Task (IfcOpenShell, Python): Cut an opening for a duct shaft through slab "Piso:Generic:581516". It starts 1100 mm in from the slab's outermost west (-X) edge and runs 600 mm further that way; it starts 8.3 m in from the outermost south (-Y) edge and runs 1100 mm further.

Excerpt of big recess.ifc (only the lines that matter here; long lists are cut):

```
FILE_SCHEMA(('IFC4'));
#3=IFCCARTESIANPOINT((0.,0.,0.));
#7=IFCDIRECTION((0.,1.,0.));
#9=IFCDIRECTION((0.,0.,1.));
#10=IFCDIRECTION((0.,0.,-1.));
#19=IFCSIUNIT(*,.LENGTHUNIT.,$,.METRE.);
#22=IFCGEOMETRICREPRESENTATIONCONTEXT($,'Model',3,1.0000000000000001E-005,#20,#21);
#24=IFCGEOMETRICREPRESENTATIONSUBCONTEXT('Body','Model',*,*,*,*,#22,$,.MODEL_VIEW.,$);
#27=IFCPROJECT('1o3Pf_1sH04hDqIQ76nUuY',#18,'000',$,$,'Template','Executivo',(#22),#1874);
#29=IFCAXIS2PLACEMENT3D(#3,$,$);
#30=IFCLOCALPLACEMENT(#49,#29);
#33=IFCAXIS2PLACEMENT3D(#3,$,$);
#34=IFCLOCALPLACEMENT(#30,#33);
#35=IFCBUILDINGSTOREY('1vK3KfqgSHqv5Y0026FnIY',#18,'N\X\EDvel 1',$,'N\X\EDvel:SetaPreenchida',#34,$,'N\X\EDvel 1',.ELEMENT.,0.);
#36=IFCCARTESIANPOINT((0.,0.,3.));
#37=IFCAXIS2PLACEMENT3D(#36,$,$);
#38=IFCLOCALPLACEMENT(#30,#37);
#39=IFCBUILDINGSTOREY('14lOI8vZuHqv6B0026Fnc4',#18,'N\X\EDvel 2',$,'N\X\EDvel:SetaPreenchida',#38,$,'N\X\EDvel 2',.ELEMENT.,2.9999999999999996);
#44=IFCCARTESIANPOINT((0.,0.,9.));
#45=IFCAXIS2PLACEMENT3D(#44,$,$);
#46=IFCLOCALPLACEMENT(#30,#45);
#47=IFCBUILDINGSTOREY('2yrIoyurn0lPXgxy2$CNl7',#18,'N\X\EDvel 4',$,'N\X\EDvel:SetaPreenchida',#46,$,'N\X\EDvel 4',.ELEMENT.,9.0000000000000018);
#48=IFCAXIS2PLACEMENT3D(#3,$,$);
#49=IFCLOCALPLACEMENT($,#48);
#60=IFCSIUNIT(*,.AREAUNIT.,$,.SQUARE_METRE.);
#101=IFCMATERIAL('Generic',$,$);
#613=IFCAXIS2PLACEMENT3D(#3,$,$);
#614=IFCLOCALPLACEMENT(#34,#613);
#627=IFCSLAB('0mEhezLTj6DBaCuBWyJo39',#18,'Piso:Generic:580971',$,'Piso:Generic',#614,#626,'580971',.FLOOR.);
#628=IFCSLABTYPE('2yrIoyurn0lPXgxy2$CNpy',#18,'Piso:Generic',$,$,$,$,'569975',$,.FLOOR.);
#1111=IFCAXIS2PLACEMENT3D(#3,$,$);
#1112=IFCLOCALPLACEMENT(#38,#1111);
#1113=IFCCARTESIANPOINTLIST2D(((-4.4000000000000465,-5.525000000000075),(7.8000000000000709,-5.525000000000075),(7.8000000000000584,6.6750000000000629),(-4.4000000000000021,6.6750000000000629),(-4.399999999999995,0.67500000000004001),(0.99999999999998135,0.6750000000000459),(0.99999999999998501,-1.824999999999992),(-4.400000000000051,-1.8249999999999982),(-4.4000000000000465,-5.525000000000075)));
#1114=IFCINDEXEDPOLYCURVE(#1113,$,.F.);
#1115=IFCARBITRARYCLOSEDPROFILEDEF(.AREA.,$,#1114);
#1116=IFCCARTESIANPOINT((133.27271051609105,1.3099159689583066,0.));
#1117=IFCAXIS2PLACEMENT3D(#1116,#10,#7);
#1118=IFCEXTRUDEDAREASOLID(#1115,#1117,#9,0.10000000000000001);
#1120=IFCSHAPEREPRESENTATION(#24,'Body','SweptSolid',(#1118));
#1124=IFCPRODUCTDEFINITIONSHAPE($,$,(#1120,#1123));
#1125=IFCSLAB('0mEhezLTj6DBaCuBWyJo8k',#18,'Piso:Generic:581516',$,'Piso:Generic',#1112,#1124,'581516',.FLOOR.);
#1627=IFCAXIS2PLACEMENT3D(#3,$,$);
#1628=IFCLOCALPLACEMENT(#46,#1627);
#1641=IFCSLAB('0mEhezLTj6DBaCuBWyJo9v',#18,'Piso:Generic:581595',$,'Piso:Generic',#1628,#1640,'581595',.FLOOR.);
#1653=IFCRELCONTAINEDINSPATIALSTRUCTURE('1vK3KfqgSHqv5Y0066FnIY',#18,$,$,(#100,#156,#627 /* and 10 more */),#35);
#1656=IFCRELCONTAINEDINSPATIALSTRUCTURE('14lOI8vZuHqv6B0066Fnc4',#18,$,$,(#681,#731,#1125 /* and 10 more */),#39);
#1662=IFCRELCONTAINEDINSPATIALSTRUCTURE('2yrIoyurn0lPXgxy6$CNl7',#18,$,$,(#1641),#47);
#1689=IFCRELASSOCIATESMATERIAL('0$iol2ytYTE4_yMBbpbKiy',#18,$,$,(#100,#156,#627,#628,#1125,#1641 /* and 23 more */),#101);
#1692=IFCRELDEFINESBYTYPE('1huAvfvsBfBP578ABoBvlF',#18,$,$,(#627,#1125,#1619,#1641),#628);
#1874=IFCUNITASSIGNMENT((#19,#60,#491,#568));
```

```python
import numpy as np
import ifcopenshell
import ifcopenshell.api.feature
import ifcopenshell.api.geometry
import ifcopenshell.api.root
import ifcopenshell.geom
import ifcopenshell.util.placement
import ifcopenshell.util.representation
import ifcopenshell.util.shape
import ifcopenshell.util.unit

model = ifcopenshell.open("big recess.ifc")
unit_scale = ifcopenshell.util.unit.calculate_unit_scale(model)
settings = ifcopenshell.geom.settings()


def volume(element):
    """Net volume in cubic metres, openings subtracted."""
    shape = ifcopenshell.geom.create_shape(settings, element)
    return ifcopenshell.util.shape.get_volume(shape.geometry)


slab = model.by_guid("0mEhezLTj6DBaCuBWyJo8k")
before = volume(slab)

# Extent in the slab's own axes, in metres. The edges named are its -X and -Y sides.
slab_shape = ifcopenshell.geom.create_shape(settings, slab)
vertices = ifcopenshell.util.shape.get_vertices(slab_shape.geometry)
x_min, y_min, bottom = vertices.min(axis=0)
top = vertices[:, 2].max()

opening = ifcopenshell.api.root.create_entity(model, ifc_class="IfcOpeningElement", name="Duct shaft opening", predefined_type="OPENING")
context = ifcopenshell.util.representation.get_context(model, "Model", "Body", "MODEL_VIEW")
width, depth = 0.6, 1.1
outline = [(0.0, 0.0), (width, 0.0), (width, depth), (0.0, depth), (0.0, 0.0)]
# Overshoot both faces by 50 mm so the cut is clean.
shape = ifcopenshell.api.geometry.add_slab_representation(
    model, context=context, depth=top - bottom + 0.1, polyline=outline
)
ifcopenshell.api.geometry.assign_representation(model, product=opening, representation=shape)

matrix = ifcopenshell.util.placement.get_local_placement(slab.ObjectPlacement)
matrix[:, 3] = matrix @ np.append(np.array([x_min + 1.1, y_min + 8.3, bottom - 0.05]) / unit_scale, 1.0)
ifcopenshell.api.geometry.edit_object_placement(model, product=opening, matrix=matrix, is_si=False)
ifcopenshell.api.feature.add_feature(model, feature=opening, element=slab)

after = volume(slab)

print(f"slab volume {before:.3f} -> {after:.3f} m3")

model.write("big recess_rev.ifc")
```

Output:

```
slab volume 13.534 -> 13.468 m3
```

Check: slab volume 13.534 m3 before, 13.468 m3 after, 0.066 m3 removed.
